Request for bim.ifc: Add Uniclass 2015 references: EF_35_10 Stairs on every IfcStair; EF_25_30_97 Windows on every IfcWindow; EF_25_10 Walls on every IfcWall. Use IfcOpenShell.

First a look at what the model holds.

```python
import ifcopenshell

model = ifcopenshell.open("bim.ifc")
print(model.schema)
print("classifications:", [c.Name for c in model.by_type("IfcClassification")])
for ifc_class in ("IfcDoor", "IfcRoof", "IfcStair", "IfcWall", "IfcWindow"):
    print(ifc_class, len(model.by_type(ifc_class)))
```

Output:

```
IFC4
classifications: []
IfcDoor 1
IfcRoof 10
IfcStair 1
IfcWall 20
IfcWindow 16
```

```python
import ifcopenshell
import ifcopenshell.api.classification

model = ifcopenshell.open("bim.ifc")

system = ifcopenshell.api.classification.add_classification(model, classification="Uniclass 2015")

codes = {
    "IfcStair": ("EF_35_10", "Stairs"),
    "IfcWindow": ("EF_25_30_97", "Windows"),
    "IfcWall": ("EF_25_10", "Walls"),
}
for ifc_class, (code, name) in codes.items():
    products = model.by_type(ifc_class)
    ifcopenshell.api.classification.add_reference(
        model, products=products, classification=system, identification=code, name=name
    )
    print(code, len(products))

model.write("bim_rev.ifc")
```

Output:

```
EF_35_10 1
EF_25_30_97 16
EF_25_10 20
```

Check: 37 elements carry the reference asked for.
